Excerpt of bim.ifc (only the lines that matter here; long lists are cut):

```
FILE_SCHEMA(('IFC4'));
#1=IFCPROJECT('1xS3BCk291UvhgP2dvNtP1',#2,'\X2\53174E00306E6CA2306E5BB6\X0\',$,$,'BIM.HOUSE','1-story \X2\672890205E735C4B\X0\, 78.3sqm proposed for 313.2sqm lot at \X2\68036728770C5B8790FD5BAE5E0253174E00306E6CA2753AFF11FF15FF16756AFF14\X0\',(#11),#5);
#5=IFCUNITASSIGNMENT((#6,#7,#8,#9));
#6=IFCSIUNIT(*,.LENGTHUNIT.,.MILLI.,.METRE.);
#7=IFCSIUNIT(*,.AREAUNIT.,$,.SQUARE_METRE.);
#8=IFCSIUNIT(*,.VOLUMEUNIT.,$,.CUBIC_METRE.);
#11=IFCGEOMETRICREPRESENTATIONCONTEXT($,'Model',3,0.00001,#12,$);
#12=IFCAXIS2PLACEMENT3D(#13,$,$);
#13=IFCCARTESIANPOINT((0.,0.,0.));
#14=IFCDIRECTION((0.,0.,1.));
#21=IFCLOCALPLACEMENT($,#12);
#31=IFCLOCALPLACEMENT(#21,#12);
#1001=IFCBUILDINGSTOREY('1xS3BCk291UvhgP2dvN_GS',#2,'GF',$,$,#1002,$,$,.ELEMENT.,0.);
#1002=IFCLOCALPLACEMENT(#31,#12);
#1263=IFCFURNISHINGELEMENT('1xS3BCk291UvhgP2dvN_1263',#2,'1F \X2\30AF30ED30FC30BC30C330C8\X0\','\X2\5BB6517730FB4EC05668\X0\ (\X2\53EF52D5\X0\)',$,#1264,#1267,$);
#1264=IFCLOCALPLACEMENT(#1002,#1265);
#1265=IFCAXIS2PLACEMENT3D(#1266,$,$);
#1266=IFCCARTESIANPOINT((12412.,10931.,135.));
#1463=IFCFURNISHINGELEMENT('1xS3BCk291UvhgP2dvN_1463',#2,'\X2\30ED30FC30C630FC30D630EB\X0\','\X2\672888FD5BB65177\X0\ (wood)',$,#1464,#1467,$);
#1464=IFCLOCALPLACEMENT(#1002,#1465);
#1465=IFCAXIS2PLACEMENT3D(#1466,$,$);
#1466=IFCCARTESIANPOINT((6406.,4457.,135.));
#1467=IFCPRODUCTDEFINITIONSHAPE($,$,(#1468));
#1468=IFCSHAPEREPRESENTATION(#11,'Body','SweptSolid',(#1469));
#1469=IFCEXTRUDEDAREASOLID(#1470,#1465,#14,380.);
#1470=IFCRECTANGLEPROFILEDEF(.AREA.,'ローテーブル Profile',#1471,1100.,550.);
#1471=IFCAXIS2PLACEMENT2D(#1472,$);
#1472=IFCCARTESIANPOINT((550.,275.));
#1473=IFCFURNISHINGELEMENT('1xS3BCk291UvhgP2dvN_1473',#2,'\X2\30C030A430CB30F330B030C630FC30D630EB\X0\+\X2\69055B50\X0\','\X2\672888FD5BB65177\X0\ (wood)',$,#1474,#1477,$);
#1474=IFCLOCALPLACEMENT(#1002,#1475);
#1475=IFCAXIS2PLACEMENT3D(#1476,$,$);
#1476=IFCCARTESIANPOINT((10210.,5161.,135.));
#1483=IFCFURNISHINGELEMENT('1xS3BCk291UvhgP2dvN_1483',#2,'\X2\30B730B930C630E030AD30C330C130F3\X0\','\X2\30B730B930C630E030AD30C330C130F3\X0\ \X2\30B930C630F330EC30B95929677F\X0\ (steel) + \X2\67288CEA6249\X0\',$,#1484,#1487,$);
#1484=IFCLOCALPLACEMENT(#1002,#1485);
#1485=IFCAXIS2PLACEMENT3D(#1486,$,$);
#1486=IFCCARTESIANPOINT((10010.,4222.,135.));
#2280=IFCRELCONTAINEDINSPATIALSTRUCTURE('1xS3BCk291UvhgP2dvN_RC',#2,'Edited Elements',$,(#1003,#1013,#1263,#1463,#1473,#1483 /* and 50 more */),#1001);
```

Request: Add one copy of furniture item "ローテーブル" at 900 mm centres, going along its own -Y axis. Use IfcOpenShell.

```python
import ifcopenshell
import ifcopenshell.api.geometry
import ifcopenshell.api.root
import ifcopenshell.util.element
import ifcopenshell.util.placement

model = ifcopenshell.open("bim.ifc")


def reuse_history(source, copy):
    """copy_class also copies each property set's owner history, people and application; keep the originals."""
    for rel in copy.IsDefinedBy:
        if rel.is_a("IfcRelDefinesByProperties") and (history := rel.RelatingPropertyDefinition.OwnerHistory):
            rel.RelatingPropertyDefinition.OwnerHistory = source.OwnerHistory
            ifcopenshell.util.element.remove_deep2(model, history)


source = model.by_guid("1xS3BCk291UvhgP2dvN_1463")
base = ifcopenshell.util.placement.get_local_placement(source.ObjectPlacement)
step = -base[:3, 1] * 900.0

for i in range(1, 2):
    copy = ifcopenshell.api.root.copy_class(model, product=source)
    copy.Representation = ifcopenshell.util.element.copy_deep(
        model, source.Representation, exclude=["IfcGeometricRepresentationContext", "IfcRepresentationMap"]
    )
    reuse_history(source, copy)
    matrix = base.copy()
    matrix[:3, 3] += i * step
    print("added at", matrix[:3, 3].round(3) + 0.0)
    ifcopenshell.api.geometry.edit_object_placement(model, product=copy, matrix=matrix, is_si=False)

model.write("bim_v2.ifc")
```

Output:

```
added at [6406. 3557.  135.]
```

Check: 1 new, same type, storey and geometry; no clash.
